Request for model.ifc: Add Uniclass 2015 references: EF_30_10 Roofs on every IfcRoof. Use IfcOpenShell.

First a look at what the model holds.

```python
import ifcopenshell

model = ifcopenshell.open("model.ifc")
print(model.schema)
print("classifications:", [c.Name for c in model.by_type("IfcClassification")])
for ifc_class in ("IfcDoor", "IfcRoof", "IfcStair", "IfcWall", "IfcWindow"):
    print(ifc_class, len(model.by_type(ifc_class)))
```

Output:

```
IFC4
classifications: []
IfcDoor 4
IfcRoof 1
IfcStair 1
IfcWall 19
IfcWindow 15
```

```python
import ifcopenshell
import ifcopenshell.api.classification

model = ifcopenshell.open("model.ifc")

system = ifcopenshell.api.classification.add_classification(model, classification="Uniclass 2015")

codes = {
    "IfcRoof": ("EF_30_10", "Roofs"),
}
for ifc_class, (code, name) in codes.items():
    products = model.by_type(ifc_class)
    ifcopenshell.api.classification.add_reference(
        model, products=products, classification=system, identification=code, name=name
    )
    print(code, len(products))

model.write("model-out.ifc")
```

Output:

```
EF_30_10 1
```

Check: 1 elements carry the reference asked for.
